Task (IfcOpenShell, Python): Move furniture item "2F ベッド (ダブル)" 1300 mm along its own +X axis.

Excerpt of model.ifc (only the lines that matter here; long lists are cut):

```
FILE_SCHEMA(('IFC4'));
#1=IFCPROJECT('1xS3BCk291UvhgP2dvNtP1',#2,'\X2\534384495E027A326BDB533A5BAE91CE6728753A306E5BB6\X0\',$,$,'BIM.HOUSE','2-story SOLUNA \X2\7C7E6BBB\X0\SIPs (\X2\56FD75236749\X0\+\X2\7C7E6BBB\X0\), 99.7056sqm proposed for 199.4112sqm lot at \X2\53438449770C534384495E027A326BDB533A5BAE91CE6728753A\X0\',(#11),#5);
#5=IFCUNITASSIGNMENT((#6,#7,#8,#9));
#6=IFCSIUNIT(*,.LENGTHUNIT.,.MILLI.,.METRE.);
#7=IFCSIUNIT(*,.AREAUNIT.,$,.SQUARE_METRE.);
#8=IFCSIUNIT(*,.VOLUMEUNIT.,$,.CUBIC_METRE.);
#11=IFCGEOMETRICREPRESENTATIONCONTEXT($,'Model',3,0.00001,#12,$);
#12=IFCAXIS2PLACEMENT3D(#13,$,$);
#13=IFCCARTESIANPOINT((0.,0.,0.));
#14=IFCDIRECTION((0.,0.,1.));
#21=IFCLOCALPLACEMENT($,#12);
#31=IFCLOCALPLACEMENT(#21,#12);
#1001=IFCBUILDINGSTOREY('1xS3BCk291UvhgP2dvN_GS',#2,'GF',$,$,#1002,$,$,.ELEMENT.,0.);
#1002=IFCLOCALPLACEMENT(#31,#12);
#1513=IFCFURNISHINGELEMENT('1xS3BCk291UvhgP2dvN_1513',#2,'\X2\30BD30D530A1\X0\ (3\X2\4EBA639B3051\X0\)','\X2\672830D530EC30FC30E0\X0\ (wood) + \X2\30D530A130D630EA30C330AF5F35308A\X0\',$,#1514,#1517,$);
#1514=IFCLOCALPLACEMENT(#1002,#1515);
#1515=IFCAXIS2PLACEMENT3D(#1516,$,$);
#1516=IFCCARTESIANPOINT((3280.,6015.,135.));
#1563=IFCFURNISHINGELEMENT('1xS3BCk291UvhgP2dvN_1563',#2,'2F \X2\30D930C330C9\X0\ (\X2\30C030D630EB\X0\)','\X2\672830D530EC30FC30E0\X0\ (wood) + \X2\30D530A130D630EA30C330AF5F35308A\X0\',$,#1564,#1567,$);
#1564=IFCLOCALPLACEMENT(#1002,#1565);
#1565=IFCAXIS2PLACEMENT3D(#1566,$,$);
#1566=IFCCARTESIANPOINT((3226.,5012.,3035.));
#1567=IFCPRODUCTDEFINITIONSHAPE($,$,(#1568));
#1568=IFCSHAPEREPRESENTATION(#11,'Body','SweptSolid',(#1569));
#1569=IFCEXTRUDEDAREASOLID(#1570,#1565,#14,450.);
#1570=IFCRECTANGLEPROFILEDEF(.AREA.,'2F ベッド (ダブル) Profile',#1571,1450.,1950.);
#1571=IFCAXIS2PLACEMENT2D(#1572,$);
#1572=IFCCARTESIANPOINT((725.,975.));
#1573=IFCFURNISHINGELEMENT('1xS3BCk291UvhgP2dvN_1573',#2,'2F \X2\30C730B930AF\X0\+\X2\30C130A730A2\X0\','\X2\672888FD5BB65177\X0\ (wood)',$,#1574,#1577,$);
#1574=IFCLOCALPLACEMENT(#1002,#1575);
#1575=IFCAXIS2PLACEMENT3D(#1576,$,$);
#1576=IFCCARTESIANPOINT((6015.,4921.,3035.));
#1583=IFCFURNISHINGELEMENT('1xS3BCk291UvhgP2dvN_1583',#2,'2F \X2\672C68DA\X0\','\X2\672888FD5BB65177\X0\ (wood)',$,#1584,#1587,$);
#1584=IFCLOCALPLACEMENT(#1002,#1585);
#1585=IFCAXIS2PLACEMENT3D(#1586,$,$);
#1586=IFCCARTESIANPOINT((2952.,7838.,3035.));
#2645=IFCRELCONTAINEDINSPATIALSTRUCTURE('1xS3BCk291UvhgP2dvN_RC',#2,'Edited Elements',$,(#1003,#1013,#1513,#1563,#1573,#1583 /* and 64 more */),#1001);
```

```python
import ifcopenshell
import ifcopenshell.api.geometry
import ifcopenshell.util.placement
import ifcopenshell.util.unit

model = ifcopenshell.open("model.ifc")
unit_scale = ifcopenshell.util.unit.calculate_unit_scale(model)

item = model.by_guid("1xS3BCk291UvhgP2dvN_1563")
matrix = ifcopenshell.util.placement.get_local_placement(item.ObjectPlacement)
matrix[:3, 3] += matrix[:3, 0] * 1.3 / unit_scale
ifcopenshell.api.geometry.edit_object_placement(model, product=item, matrix=matrix, is_si=False)

print(ifcopenshell.util.placement.get_local_placement(item.ObjectPlacement).round(3) + 0.0)

model.write("model-out.ifc")
```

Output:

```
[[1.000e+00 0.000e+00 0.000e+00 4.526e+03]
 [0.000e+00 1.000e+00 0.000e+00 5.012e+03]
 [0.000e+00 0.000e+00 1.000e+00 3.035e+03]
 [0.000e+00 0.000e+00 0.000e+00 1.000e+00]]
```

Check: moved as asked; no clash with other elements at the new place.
